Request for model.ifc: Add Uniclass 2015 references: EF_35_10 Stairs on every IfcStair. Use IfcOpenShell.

First a look at what the model holds.

```python
import ifcopenshell

model = ifcopenshell.open("model.ifc")
print(model.schema)
print("classifications:", [c.Name for c in model.by_type("IfcClassification")])
for ifc_class in ("IfcDoor", "IfcRoof", "IfcStair", "IfcWall", "IfcWindow"):
    print(ifc_class, len(model.by_type(ifc_class)))
```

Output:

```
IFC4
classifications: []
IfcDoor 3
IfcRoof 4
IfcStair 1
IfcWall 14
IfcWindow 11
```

```python
import ifcopenshell
import ifcopenshell.api.classification

model = ifcopenshell.open("model.ifc")

system = ifcopenshell.api.classification.add_classification(model, classification="Uniclass 2015")

codes = {
    "IfcStair": ("EF_35_10", "Stairs"),
}
for ifc_class, (code, name) in codes.items():
    products = model.by_type(ifc_class)
    ifcopenshell.api.classification.add_reference(
        model, products=products, classification=system, identification=code, name=name
    )
    print(code, len(products))

model.write("model_rev.ifc")
```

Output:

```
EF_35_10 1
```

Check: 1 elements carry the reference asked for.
